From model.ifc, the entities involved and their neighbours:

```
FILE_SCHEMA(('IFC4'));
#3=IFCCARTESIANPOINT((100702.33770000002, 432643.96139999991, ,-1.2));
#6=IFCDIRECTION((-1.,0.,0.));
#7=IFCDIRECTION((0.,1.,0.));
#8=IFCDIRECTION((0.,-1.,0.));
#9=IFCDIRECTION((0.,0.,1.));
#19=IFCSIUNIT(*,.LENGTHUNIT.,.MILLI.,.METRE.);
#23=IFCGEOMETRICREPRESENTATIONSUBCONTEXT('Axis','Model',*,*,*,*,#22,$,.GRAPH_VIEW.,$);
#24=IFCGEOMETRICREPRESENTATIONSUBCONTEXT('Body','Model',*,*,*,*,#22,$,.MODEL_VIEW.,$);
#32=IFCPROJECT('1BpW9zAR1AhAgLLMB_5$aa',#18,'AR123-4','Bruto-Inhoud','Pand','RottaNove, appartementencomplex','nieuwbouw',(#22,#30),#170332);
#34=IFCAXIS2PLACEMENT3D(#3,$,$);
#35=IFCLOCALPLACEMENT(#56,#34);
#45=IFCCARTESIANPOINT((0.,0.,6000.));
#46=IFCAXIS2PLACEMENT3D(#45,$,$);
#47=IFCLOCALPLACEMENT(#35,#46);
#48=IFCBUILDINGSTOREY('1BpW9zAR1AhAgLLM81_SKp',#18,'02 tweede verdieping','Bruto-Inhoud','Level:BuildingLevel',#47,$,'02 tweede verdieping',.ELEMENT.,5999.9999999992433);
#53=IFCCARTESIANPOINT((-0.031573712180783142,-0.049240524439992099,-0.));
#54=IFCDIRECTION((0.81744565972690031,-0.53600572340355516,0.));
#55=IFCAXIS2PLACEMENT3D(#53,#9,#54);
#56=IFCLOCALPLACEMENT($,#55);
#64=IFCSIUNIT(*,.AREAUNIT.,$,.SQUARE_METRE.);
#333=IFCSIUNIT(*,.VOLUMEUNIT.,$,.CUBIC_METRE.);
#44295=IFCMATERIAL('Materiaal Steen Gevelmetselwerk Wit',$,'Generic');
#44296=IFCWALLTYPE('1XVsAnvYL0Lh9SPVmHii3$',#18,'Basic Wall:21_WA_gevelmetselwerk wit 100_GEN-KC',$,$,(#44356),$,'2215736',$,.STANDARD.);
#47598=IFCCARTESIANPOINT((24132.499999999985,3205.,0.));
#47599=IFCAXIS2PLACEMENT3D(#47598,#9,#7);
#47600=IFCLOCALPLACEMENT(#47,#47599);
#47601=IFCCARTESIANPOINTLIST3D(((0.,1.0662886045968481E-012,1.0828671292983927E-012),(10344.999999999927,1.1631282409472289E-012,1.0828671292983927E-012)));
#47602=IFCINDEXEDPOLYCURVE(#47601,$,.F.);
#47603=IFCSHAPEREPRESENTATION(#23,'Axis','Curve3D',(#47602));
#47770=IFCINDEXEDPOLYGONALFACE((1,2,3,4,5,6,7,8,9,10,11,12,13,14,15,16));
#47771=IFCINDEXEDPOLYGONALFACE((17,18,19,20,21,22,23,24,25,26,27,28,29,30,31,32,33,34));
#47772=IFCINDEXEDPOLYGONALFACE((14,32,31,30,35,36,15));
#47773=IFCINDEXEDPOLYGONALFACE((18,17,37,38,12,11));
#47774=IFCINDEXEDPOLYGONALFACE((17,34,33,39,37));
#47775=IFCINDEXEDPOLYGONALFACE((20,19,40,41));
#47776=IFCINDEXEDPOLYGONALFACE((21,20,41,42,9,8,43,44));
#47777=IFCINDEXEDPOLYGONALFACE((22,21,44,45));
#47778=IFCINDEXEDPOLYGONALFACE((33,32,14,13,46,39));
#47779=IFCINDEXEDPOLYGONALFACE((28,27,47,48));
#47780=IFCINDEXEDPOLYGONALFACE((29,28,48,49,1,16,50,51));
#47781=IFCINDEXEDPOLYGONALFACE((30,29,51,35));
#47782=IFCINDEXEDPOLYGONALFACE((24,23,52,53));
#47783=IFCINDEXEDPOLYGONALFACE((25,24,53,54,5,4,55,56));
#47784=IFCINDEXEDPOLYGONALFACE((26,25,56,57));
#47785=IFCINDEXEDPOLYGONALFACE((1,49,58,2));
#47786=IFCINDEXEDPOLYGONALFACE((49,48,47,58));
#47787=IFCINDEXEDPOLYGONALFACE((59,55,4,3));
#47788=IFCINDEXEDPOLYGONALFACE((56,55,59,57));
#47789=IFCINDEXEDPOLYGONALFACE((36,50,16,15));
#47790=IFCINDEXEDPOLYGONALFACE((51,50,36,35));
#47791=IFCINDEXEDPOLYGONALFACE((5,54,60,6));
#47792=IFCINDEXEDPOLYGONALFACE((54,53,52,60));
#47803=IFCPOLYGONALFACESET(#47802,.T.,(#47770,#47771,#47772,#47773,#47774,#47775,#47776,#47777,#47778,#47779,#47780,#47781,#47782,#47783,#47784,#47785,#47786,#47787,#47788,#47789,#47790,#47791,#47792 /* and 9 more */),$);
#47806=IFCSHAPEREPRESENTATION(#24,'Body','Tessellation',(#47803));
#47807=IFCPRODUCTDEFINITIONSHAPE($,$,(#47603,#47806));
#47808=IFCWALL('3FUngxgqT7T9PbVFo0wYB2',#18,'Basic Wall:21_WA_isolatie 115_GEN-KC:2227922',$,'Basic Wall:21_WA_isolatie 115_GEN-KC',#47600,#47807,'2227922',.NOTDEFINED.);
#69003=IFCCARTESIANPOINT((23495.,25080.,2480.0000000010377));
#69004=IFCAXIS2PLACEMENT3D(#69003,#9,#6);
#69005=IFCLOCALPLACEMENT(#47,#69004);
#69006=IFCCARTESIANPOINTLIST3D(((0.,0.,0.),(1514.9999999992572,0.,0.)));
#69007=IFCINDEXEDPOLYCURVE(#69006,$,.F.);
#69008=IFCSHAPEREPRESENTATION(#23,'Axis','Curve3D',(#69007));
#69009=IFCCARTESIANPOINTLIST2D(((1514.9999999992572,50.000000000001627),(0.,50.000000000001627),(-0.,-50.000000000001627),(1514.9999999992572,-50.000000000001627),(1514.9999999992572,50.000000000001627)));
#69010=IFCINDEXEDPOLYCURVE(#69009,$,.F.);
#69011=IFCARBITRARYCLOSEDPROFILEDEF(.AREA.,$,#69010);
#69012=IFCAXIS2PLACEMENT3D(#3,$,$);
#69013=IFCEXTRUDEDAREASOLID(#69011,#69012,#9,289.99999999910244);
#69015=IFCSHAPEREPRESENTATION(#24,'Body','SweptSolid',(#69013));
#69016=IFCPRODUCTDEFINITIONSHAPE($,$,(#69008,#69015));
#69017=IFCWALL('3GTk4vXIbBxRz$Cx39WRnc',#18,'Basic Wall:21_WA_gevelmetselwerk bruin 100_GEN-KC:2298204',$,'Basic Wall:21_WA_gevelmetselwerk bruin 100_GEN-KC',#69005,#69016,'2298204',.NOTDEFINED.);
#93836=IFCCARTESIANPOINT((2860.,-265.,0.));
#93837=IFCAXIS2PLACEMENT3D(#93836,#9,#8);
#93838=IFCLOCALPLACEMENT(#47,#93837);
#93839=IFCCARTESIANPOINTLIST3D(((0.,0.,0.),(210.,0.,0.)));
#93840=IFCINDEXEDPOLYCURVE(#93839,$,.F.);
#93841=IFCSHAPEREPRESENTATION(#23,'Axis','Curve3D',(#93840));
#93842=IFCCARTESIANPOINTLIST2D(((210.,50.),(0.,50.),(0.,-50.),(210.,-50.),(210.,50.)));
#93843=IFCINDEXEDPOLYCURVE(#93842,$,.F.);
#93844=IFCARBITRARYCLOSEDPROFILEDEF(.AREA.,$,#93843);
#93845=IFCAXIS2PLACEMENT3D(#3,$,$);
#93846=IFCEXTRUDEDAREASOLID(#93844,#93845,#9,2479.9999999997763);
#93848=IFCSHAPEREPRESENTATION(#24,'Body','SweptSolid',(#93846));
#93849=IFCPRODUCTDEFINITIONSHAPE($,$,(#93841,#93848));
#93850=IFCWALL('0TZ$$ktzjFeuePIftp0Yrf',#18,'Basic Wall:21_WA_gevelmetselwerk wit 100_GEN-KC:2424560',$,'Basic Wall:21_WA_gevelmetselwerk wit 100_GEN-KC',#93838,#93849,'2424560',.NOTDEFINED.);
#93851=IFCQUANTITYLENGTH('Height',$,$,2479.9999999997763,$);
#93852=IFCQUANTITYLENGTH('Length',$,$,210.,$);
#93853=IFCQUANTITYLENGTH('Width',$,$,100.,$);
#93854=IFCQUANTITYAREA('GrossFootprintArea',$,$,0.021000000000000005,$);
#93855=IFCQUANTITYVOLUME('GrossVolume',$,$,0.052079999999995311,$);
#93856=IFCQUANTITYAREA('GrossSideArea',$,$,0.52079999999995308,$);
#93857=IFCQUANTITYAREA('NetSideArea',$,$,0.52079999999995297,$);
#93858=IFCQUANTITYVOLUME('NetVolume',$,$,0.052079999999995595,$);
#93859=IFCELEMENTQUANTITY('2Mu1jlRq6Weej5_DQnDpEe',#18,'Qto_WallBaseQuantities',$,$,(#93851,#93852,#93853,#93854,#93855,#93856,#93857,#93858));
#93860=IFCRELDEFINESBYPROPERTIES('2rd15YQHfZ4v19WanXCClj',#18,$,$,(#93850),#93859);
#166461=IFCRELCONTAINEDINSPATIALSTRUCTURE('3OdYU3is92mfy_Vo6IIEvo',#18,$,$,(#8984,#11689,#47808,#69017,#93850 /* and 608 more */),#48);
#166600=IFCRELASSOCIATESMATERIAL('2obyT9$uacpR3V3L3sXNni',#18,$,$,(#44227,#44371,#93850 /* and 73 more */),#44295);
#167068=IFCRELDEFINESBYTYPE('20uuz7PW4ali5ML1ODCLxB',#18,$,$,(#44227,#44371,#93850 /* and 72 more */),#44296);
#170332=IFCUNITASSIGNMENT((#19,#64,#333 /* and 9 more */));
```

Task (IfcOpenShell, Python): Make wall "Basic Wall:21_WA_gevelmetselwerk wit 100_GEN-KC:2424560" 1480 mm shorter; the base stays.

```python
import ifcopenshell
import ifcopenshell.api.pset
import ifcopenshell.geom
import ifcopenshell.util.element
import ifcopenshell.util.representation
import ifcopenshell.util.shape
import ifcopenshell.util.unit

model = ifcopenshell.open("model.ifc")
unit_scale = ifcopenshell.util.unit.calculate_unit_scale(model)
area_scale = ifcopenshell.util.unit.calculate_unit_scale(model, "AREAUNIT")
volume_scale = ifcopenshell.util.unit.calculate_unit_scale(model, "VOLUMEUNIT")
settings = ifcopenshell.geom.settings()


def volume(element):
    """Net volume in cubic metres, openings subtracted."""
    shape = ifcopenshell.geom.create_shape(settings, element)
    return ifcopenshell.util.shape.get_volume(shape.geometry)


wall = model.by_guid("0TZ$$ktzjFeuePIftp0Yrf")
before = volume(wall)

body = ifcopenshell.util.representation.get_representation(wall, "Model", "Body")
solid = body.Items[0]
old_height = solid.Depth
solid.Depth -= 1.48 / unit_scale
after = volume(wall)
thickness = 0.1  # wall thickness in metres

# Update the stored height, areas and volumes.
qto = model.by_id(ifcopenshell.util.element.get_pset(wall, "Qto_WallBaseQuantities", should_inherit=False)["id"])
ifcopenshell.api.pset.edit_qto(model, qto=qto, properties={
    "Height": solid.Depth,
    "GrossVolume": ifcopenshell.util.element.get_pset(wall, "Qto_WallBaseQuantities", "GrossVolume") * solid.Depth / old_height,
    "GrossSideArea": ifcopenshell.util.element.get_pset(wall, "Qto_WallBaseQuantities", "GrossSideArea") * solid.Depth / old_height,
    "NetSideArea": after / thickness / area_scale,
    "NetVolume": after / volume_scale,
})

print(f"height {old_height:g} -> {solid.Depth:g}, volume {before:.3f} -> {after:.3f} m3")

model.write("model_v2.ifc")
```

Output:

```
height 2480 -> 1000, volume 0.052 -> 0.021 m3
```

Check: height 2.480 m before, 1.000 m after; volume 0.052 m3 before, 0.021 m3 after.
